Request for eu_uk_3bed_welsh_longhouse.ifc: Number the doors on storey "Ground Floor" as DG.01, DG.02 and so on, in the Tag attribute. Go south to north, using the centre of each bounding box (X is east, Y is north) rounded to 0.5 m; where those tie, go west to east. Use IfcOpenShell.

First a look at what the model holds.

```python
import ifcopenshell
import ifcopenshell.util.element
import ifcopenshell.util.placement

model = ifcopenshell.open("eu_uk_3bed_welsh_longhouse.ifc")
print(model.schema)
storey = next(s for s in model.by_type("IfcBuildingStorey") if s.Name == "Ground Floor")
doors = [e for e in ifcopenshell.util.element.get_decomposition(storey) if e.is_a("IfcDoor")]
for e in sorted(doors, key=lambda e: e.id()):
    origin = ifcopenshell.util.placement.get_local_placement(e.ObjectPlacement)[:3, 3]
    print(e.id(), e.Tag, e.Name, origin.round(2) + 0.0, sep=" | ")
```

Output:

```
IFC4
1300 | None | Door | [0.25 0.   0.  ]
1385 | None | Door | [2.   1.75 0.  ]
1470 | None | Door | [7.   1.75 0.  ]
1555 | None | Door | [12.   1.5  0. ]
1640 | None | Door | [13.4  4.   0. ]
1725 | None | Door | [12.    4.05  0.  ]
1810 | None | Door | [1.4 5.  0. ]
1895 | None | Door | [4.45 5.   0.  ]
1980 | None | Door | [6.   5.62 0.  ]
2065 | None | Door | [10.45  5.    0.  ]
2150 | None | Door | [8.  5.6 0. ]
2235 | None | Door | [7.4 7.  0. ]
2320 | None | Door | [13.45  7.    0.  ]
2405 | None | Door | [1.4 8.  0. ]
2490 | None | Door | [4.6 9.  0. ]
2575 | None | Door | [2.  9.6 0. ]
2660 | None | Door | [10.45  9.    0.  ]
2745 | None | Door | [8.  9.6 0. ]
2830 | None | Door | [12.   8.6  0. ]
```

```python
import ifcopenshell
import ifcopenshell.geom
import ifcopenshell.util.element
import ifcopenshell.util.shape

model = ifcopenshell.open("eu_uk_3bed_welsh_longhouse.ifc")
settings = ifcopenshell.geom.settings()
settings.set("use-world-coords", True)


def centre(element):
    shape = ifcopenshell.geom.create_shape(settings, element)
    return ifcopenshell.util.shape.get_bbox_centroid(shape.geometry)


storey = next(s for s in model.by_type("IfcBuildingStorey") if s.Name == "Ground Floor")
doors = [e for e in ifcopenshell.util.element.get_decomposition(storey) if e.is_a("IfcDoor")]

# Insertion points can sit at a corner or the storey origin, so sort by the geometry (in metres).
centres = {e: centre(e) for e in doors}
doors.sort(key=lambda e: (round(centres[e][1] / 0.5), centres[e][0]))

for i, e in enumerate(doors, start=1):
    number = f"DG.{i:02d}"
    e.Tag = number
    print(e.id(), number)

model.write("eu_uk_3bed_welsh_longhouse_rev.ifc")
```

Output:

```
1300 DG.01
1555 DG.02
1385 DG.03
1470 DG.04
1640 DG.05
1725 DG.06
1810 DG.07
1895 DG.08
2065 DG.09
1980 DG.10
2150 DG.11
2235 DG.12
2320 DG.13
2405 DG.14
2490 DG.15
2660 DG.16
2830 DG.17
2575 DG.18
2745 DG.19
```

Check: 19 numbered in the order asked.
